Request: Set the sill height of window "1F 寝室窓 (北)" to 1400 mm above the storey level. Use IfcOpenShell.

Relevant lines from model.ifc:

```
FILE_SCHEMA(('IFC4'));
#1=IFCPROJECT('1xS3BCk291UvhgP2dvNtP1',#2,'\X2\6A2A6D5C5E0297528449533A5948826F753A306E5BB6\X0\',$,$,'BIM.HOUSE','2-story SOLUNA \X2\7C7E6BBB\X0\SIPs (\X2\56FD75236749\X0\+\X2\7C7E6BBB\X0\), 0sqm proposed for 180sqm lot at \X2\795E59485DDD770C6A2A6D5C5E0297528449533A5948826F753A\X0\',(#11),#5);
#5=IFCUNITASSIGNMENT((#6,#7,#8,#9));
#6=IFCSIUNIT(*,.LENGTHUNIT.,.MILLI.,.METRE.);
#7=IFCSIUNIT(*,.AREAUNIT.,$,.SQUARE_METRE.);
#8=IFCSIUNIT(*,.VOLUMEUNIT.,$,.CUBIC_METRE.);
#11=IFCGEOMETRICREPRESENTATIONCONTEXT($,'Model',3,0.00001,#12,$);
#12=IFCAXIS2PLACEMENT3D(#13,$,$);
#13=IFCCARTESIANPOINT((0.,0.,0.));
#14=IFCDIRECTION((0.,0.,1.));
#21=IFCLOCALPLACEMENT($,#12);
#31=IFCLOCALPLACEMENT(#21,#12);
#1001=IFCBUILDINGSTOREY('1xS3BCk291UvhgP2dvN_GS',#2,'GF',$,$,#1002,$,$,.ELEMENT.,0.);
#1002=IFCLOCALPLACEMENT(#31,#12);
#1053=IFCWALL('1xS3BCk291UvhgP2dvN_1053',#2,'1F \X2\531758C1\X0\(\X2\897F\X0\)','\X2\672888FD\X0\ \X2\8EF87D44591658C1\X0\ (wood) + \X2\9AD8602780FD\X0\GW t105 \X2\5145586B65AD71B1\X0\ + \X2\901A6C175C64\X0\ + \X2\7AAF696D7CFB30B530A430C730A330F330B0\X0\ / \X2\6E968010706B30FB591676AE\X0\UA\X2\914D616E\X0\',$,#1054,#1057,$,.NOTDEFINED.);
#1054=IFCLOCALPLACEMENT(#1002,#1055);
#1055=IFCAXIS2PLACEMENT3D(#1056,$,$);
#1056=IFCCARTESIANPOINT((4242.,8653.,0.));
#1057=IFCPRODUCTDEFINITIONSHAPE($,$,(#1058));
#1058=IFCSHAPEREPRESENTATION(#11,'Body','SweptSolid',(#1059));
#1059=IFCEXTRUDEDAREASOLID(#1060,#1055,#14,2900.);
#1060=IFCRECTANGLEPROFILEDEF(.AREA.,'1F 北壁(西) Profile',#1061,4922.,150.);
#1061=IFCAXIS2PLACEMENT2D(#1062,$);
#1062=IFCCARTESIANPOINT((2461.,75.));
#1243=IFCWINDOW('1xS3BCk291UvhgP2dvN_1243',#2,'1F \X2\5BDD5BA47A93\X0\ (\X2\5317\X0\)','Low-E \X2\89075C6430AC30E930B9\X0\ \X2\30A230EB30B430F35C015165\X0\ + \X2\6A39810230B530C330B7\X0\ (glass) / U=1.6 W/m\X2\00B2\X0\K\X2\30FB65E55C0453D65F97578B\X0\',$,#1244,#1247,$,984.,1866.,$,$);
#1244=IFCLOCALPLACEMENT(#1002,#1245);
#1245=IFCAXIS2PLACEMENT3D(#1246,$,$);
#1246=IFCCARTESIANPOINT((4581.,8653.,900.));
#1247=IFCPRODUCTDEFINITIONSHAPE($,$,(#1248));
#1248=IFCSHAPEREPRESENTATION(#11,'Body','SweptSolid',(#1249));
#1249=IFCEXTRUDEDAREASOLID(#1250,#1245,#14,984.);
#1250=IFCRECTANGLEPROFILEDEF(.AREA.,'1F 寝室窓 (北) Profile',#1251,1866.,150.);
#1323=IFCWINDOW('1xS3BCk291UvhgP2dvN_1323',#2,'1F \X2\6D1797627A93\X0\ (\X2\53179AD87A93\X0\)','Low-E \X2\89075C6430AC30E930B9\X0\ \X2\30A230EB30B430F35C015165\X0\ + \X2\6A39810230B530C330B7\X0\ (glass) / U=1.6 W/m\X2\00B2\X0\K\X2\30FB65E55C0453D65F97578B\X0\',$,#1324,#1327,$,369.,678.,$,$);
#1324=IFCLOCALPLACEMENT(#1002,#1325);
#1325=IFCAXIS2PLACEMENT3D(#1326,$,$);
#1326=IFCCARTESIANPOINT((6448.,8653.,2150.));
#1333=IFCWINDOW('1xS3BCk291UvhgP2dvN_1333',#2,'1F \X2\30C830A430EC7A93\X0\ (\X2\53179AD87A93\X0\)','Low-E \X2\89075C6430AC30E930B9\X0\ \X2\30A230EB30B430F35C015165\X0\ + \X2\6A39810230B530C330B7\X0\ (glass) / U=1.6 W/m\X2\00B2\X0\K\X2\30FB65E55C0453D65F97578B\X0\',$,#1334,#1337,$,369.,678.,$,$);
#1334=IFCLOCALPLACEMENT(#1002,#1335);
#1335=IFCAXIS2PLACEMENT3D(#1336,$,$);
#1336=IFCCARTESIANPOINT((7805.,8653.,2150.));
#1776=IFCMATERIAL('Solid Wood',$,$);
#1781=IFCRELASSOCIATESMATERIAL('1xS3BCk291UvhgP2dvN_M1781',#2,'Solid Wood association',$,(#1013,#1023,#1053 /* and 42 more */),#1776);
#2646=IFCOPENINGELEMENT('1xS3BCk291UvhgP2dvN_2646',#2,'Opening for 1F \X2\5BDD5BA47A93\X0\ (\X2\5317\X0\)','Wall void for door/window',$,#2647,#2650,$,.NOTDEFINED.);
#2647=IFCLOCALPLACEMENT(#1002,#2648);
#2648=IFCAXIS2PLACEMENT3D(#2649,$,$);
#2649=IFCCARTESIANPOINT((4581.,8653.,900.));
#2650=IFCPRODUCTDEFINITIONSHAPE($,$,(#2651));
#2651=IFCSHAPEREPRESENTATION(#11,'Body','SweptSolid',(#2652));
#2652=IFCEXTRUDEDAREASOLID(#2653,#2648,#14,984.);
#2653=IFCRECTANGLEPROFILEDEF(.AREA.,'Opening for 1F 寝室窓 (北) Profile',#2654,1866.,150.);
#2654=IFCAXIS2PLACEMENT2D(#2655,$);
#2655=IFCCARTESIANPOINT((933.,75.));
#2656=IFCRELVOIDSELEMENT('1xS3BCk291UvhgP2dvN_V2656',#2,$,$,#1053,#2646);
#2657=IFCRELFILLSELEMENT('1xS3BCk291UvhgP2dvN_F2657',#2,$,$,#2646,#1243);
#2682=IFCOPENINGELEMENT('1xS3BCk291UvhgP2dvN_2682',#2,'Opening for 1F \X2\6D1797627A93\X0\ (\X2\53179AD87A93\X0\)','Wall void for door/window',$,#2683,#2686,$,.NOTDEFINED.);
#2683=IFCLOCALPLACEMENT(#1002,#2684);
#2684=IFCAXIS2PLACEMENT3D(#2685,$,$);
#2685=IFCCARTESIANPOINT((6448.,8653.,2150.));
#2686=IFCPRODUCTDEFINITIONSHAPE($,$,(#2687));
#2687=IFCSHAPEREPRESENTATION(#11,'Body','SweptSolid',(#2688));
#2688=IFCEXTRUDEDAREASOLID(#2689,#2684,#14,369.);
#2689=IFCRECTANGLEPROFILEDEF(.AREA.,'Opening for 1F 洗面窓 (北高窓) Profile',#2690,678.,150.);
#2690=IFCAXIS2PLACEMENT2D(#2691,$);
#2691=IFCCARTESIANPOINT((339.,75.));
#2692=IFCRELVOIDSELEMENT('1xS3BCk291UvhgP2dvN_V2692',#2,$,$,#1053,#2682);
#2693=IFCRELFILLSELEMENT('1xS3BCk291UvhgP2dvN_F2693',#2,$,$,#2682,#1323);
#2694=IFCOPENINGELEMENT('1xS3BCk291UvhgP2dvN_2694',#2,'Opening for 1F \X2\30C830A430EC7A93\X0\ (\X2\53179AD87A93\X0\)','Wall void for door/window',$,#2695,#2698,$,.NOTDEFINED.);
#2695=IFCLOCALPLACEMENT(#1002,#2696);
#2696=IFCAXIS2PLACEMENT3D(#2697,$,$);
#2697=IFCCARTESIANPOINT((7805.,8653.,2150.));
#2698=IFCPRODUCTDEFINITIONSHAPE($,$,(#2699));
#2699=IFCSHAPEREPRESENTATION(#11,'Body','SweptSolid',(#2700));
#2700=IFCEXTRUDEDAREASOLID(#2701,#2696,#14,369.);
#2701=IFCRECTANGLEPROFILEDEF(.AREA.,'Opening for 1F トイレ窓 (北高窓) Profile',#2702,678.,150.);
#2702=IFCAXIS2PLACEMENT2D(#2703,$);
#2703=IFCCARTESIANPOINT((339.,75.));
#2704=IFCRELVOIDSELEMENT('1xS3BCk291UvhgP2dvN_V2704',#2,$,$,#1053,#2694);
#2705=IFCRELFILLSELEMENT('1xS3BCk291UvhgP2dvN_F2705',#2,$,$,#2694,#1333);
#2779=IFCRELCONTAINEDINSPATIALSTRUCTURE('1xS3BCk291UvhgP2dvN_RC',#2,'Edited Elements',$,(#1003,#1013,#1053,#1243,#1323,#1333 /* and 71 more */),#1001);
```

```python
import numpy as np
import ifcopenshell
import ifcopenshell.api.geometry
import ifcopenshell.geom
import ifcopenshell.util.element
import ifcopenshell.util.placement
import ifcopenshell.util.shape
import ifcopenshell.util.unit

model = ifcopenshell.open("model.ifc")
unit_scale = ifcopenshell.util.unit.calculate_unit_scale(model)

window = model.by_id(1243)
opening = window.FillsVoids[0].RelatingOpeningElement
storey = ifcopenshell.util.element.get_container(window, ifc_class="IfcBuildingStorey")
level = ifcopenshell.util.placement.get_local_placement(storey.ObjectPlacement)[2, 3]

# The opening's origin need not be at the sill, so measure its lowest point.
shape = ifcopenshell.geom.create_shape(ifcopenshell.geom.settings(), opening)
bottom = ifcopenshell.util.shape.get_shape_bottom_elevation(shape, shape.geometry) / unit_scale
dz = level + 1.4 / unit_scale - bottom

shift = np.array([0.0, 0.0, dz])
# The window is not placed relative to its opening, so move both.
for product in (opening, window):
    matrix = ifcopenshell.util.placement.get_local_placement(product.ObjectPlacement)
    matrix[:3, 3] += shift
    ifcopenshell.api.geometry.edit_object_placement(model, product=product, matrix=matrix, is_si=False)

print(f"moved by {dz * unit_scale:+.3f} m")

model.write("model_rev.ifc")
```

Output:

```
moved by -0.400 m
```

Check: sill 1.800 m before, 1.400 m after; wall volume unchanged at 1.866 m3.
